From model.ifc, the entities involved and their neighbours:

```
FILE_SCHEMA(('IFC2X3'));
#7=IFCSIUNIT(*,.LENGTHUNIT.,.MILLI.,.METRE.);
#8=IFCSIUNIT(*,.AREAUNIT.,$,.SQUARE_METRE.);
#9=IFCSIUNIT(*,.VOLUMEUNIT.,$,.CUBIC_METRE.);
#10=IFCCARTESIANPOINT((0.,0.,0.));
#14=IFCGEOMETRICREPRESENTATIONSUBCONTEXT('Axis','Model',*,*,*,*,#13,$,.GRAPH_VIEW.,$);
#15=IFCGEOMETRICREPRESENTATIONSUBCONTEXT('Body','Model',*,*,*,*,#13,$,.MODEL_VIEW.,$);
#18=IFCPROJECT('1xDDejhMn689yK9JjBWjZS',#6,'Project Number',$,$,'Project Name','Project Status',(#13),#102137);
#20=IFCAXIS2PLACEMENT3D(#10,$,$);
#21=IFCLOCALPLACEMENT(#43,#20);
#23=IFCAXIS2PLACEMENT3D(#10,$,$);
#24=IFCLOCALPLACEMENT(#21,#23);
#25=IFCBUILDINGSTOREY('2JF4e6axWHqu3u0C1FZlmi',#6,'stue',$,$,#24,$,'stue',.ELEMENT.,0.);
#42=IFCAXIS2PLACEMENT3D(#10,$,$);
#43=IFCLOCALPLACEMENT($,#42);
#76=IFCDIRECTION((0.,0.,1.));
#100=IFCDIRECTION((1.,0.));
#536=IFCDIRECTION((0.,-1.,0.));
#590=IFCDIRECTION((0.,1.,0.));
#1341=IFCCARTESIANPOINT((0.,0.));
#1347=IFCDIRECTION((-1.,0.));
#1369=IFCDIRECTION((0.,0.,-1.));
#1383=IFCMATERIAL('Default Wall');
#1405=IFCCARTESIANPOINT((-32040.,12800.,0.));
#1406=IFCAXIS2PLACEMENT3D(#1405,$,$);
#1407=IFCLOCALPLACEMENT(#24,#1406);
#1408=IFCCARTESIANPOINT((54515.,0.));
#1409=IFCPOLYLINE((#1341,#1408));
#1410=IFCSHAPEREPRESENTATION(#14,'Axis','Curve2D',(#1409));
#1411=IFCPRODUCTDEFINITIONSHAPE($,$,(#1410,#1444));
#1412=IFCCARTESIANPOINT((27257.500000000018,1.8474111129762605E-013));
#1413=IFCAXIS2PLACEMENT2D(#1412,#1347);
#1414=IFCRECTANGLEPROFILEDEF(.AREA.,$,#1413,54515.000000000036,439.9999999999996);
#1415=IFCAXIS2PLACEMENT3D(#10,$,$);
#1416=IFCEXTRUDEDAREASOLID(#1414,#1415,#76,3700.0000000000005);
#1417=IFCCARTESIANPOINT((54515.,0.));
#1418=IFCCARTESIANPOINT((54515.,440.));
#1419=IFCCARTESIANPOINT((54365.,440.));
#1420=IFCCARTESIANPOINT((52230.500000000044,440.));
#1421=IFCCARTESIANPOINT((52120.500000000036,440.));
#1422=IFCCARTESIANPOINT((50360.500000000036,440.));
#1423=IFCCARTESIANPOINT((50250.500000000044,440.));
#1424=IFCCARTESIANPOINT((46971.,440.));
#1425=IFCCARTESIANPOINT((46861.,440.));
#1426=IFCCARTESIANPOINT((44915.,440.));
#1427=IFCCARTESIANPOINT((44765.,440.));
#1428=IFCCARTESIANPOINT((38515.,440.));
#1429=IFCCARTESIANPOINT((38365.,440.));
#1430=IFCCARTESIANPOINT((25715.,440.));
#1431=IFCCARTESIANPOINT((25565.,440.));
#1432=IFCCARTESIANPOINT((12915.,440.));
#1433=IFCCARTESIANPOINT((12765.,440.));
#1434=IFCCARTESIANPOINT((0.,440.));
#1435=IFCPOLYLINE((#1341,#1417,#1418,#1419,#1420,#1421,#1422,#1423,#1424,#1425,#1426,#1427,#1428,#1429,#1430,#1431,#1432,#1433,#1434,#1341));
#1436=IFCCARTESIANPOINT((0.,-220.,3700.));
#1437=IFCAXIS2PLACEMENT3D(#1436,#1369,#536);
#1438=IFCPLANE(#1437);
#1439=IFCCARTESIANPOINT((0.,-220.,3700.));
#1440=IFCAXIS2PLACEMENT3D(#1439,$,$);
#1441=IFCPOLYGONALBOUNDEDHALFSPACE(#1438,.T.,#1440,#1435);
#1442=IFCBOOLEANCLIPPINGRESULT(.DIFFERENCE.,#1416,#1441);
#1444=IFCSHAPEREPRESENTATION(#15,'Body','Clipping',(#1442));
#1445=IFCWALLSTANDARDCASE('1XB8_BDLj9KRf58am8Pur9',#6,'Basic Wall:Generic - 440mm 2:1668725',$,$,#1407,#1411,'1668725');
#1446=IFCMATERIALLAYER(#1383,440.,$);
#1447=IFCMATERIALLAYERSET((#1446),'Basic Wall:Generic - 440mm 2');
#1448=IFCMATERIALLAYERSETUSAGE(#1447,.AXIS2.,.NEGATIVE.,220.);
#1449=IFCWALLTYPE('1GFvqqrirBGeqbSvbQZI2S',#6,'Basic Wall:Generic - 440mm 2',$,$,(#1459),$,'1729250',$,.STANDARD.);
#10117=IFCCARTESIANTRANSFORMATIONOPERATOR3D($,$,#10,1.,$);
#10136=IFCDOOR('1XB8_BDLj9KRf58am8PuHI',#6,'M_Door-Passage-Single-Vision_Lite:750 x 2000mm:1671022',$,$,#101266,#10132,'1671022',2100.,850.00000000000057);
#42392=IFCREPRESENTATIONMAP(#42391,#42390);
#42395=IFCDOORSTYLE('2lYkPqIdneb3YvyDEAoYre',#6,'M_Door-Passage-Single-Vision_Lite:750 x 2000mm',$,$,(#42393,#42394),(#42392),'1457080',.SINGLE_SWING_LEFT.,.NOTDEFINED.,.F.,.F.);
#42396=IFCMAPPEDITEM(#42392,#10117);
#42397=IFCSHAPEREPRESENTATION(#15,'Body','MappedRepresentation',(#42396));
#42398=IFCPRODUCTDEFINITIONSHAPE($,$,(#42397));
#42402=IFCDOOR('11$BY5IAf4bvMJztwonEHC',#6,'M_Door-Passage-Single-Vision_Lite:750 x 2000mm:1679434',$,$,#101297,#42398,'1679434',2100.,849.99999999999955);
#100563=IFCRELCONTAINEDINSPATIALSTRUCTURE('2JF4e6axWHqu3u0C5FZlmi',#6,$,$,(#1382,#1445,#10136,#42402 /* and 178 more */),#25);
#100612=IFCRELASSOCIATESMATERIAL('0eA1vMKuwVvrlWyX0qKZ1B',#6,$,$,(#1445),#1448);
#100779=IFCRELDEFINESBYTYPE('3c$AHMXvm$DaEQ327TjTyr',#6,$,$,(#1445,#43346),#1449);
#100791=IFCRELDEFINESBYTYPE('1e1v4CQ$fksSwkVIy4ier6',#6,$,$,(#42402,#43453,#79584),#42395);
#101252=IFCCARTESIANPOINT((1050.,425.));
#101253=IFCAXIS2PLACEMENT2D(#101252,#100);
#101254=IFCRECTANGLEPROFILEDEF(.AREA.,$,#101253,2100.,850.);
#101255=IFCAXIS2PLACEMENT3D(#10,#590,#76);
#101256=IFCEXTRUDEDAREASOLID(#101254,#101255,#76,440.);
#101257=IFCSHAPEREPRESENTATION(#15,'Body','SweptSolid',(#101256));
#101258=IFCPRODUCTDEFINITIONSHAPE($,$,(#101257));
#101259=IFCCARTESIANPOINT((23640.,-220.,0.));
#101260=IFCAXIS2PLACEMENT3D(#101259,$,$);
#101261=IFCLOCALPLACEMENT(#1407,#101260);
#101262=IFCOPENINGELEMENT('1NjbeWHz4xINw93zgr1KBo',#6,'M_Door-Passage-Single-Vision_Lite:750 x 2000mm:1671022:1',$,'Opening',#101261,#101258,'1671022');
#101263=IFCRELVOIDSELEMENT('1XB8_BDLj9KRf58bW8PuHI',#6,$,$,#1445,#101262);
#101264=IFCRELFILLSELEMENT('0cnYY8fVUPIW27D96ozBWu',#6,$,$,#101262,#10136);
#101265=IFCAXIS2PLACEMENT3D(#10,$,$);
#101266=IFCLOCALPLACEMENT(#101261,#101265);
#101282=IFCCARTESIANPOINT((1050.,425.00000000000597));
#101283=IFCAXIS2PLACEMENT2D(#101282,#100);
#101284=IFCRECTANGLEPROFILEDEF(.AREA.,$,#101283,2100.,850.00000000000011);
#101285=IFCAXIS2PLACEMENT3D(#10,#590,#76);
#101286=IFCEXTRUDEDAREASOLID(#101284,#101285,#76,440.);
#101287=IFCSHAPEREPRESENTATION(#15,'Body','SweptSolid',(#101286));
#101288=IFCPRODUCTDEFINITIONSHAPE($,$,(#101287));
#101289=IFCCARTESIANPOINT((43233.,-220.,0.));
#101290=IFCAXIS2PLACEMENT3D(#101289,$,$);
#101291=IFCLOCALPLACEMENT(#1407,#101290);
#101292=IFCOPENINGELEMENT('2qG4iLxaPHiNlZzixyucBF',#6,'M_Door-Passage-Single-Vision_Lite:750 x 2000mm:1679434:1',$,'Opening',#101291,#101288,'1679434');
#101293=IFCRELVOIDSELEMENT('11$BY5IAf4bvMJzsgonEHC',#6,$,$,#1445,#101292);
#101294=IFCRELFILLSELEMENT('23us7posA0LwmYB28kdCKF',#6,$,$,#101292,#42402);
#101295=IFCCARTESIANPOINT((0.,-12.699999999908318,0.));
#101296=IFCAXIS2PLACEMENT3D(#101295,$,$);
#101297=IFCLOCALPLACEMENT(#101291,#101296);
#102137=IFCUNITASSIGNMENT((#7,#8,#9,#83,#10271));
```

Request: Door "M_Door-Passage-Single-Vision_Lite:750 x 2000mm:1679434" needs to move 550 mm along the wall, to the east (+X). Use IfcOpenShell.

```python
import ifcopenshell
import ifcopenshell.api.geometry
import ifcopenshell.util.placement

model = ifcopenshell.open("model.ifc")

door = model.by_guid("11$BY5IAf4bvMJztwonEHC")
opening = door.FillsVoids[0].RelatingOpeningElement
wall = opening.VoidsElements[0].RelatingBuildingElement

wall_matrix = ifcopenshell.util.placement.get_local_placement(wall.ObjectPlacement)
shift = wall_matrix[:3, 0] * 550.0
before = ifcopenshell.util.placement.get_local_placement(door.ObjectPlacement)[:3, 3].copy()

# The door is placed relative to its opening, so it follows when the opening moves.
matrix = ifcopenshell.util.placement.get_local_placement(opening.ObjectPlacement)
matrix[:3, 3] += shift
ifcopenshell.api.geometry.edit_object_placement(
    model, product=opening, matrix=matrix, is_si=False, should_transform_children=True
)

after = ifcopenshell.util.placement.get_local_placement(door.ObjectPlacement)[:3, 3]
print("door moved by", (after - before).round(3) + 0.0)

model.write("model_edited.ifc")
```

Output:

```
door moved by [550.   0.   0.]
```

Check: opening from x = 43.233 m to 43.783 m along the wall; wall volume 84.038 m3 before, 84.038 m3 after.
